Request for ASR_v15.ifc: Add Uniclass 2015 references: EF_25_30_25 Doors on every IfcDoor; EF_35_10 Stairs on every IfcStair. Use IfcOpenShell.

First a look at what the model holds.

```python
import ifcopenshell

model = ifcopenshell.open("ASR_v15.ifc")
print(model.schema)
print("classifications:", [c.Name for c in model.by_type("IfcClassification")])
for ifc_class in ("IfcDoor", "IfcRoof", "IfcStair", "IfcWall", "IfcWindow"):
    print(ifc_class, len(model.by_type(ifc_class)))
```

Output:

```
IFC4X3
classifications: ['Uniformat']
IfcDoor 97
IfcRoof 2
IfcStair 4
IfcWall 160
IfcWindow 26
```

```python
import ifcopenshell
import ifcopenshell.api.classification

model = ifcopenshell.open("ASR_v15.ifc")

system = ifcopenshell.api.classification.add_classification(model, classification="Uniclass 2015")

codes = {
    "IfcDoor": ("EF_25_30_25", "Doors"),
    "IfcStair": ("EF_35_10", "Stairs"),
}
for ifc_class, (code, name) in codes.items():
    products = model.by_type(ifc_class)
    ifcopenshell.api.classification.add_reference(
        model, products=products, classification=system, identification=code, name=name
    )
    print(code, len(products))

model.write("ASR_v15-out.ifc")
```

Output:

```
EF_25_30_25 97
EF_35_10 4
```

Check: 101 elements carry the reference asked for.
